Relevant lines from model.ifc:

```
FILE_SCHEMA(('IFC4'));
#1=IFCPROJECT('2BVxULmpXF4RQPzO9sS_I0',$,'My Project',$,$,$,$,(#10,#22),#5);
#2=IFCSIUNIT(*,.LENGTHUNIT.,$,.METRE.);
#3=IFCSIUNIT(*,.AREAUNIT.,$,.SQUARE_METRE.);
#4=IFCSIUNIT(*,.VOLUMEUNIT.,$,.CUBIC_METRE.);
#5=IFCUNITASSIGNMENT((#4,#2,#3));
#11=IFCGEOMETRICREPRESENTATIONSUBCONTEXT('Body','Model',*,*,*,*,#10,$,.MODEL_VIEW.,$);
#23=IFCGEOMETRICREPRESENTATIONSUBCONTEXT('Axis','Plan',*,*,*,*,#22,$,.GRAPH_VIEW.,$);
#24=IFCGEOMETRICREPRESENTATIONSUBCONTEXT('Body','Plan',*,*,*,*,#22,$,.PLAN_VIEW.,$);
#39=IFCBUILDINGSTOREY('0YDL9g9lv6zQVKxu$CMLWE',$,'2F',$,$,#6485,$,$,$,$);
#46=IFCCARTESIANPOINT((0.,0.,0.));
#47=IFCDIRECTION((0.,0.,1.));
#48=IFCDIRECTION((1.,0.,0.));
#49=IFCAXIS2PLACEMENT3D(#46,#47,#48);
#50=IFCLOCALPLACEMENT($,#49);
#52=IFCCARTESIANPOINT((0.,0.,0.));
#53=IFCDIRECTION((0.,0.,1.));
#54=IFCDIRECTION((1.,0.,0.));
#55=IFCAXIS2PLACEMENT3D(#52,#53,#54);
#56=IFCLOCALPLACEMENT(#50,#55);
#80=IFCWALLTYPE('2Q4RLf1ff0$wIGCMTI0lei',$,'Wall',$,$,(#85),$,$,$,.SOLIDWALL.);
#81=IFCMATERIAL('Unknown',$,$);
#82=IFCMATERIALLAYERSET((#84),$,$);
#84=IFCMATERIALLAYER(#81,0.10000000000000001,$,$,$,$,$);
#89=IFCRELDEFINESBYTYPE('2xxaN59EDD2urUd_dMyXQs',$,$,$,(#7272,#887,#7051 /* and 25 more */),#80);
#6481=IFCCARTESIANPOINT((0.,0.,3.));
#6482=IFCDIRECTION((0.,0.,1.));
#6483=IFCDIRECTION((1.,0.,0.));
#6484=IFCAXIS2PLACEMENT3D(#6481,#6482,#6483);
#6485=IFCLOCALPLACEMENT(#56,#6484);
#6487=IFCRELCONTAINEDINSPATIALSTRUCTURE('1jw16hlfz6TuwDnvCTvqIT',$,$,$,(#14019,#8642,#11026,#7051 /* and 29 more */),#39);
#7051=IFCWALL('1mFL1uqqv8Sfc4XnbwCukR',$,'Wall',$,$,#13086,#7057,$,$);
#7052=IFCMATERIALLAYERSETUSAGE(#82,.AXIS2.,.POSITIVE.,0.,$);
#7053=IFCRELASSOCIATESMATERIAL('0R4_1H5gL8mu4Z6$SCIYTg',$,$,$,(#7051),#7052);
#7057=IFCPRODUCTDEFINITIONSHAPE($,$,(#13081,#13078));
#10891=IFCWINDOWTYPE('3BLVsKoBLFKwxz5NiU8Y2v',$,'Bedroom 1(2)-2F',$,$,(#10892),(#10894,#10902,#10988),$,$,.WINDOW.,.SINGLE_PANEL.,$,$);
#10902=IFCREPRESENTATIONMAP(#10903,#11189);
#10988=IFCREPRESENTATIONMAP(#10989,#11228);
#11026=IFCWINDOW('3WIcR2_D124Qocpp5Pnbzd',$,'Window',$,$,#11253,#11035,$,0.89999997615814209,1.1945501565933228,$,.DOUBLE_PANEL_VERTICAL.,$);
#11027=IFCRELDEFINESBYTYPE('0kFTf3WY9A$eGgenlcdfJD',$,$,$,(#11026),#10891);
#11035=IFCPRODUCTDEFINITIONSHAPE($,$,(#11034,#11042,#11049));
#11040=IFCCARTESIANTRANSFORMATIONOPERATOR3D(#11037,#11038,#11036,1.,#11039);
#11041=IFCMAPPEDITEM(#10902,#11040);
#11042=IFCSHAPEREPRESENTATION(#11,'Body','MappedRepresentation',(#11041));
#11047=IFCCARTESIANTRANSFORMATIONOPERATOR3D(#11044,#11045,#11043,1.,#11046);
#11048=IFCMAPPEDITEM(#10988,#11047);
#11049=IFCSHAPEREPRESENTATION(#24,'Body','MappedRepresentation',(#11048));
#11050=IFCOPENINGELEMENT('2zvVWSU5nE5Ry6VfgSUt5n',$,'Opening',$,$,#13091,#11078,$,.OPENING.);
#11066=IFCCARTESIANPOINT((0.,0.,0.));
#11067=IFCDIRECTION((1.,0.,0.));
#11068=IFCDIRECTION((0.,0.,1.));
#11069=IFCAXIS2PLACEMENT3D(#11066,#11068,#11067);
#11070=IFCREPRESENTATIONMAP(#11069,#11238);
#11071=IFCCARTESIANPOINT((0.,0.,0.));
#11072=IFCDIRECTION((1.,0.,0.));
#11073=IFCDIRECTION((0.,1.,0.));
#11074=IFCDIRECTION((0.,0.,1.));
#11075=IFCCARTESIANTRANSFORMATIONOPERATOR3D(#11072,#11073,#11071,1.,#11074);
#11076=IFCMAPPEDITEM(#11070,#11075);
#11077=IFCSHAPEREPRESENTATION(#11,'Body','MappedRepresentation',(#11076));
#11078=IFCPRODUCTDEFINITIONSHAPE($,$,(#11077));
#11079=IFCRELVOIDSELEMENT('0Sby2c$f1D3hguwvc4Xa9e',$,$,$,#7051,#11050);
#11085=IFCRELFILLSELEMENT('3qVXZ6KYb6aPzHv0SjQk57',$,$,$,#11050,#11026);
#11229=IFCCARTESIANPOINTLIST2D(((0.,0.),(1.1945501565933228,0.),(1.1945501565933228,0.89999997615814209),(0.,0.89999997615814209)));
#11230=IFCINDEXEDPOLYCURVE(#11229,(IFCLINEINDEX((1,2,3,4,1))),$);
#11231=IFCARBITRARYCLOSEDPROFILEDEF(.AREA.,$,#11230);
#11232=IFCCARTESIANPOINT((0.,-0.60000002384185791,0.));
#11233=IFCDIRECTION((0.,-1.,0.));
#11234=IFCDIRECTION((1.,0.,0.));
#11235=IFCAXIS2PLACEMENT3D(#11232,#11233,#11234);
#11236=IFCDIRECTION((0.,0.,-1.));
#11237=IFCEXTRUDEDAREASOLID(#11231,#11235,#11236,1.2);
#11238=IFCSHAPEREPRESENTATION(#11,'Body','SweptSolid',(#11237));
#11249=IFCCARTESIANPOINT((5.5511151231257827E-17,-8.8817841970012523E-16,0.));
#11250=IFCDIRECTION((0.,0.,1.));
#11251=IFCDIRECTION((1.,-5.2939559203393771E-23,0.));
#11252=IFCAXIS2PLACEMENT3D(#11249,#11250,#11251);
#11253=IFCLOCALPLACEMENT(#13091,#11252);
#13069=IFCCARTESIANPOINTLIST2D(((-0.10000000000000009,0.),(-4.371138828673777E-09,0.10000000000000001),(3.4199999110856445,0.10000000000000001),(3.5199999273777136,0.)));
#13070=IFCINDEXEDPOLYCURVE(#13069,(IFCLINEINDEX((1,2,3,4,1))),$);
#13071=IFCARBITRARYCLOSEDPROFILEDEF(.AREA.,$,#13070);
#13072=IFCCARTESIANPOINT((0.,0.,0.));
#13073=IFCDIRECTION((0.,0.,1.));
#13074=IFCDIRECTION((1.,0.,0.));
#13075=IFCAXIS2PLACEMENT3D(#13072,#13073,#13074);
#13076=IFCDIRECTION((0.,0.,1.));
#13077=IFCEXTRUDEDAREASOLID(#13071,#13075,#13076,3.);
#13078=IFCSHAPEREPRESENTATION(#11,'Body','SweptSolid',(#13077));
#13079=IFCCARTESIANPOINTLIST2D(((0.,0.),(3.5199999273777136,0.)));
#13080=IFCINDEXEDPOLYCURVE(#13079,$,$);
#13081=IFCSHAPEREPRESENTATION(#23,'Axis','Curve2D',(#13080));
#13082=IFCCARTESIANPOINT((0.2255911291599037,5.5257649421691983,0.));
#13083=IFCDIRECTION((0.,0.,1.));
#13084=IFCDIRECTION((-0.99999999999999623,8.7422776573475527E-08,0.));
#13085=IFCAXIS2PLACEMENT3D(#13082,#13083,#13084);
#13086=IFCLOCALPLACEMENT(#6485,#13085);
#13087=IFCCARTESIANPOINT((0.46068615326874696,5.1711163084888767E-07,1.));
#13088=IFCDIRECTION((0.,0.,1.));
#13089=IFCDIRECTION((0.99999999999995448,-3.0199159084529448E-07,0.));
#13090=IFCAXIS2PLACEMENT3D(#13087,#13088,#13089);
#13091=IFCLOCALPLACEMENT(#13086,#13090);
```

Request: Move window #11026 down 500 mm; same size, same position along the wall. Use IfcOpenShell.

```python
import numpy as np
import ifcopenshell
import ifcopenshell.api.geometry
import ifcopenshell.util.placement
import ifcopenshell.util.unit

model = ifcopenshell.open("model.ifc")
unit_scale = ifcopenshell.util.unit.calculate_unit_scale(model)

window = model.by_id(11026)
opening = window.FillsVoids[0].RelatingOpeningElement
dz = -0.5 / unit_scale

shift = np.array([0.0, 0.0, dz])
# The window is placed relative to its opening, so it follows when the opening moves.
matrix = ifcopenshell.util.placement.get_local_placement(opening.ObjectPlacement)
matrix[:3, 3] += shift
ifcopenshell.api.geometry.edit_object_placement(
    model, product=opening, matrix=matrix, is_si=False, should_transform_children=True
)

print(f"moved by {dz * unit_scale:+.3f} m")

model.write("model_rev.ifc")
```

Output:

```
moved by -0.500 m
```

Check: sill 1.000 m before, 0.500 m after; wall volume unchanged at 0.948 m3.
